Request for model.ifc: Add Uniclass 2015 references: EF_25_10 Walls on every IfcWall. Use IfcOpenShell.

First a look at what the model holds.

```python
import ifcopenshell

model = ifcopenshell.open("model.ifc")
print(model.schema)
print("classifications:", [c.Name for c in model.by_type("IfcClassification")])
for ifc_class in ("IfcDoor", "IfcRoof", "IfcStair", "IfcWall", "IfcWindow"):
    print(ifc_class, len(model.by_type(ifc_class)))
```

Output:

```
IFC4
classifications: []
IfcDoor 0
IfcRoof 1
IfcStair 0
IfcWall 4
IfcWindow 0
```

```python
import ifcopenshell
import ifcopenshell.api.classification

model = ifcopenshell.open("model.ifc")

system = ifcopenshell.api.classification.add_classification(model, classification="Uniclass 2015")

codes = {
    "IfcWall": ("EF_25_10", "Walls"),
}
for ifc_class, (code, name) in codes.items():
    products = model.by_type(ifc_class)
    ifcopenshell.api.classification.add_reference(
        model, products=products, classification=system, identification=code, name=name
    )
    print(code, len(products))

model.write("model_updated.ifc")
```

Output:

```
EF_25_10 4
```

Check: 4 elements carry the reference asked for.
